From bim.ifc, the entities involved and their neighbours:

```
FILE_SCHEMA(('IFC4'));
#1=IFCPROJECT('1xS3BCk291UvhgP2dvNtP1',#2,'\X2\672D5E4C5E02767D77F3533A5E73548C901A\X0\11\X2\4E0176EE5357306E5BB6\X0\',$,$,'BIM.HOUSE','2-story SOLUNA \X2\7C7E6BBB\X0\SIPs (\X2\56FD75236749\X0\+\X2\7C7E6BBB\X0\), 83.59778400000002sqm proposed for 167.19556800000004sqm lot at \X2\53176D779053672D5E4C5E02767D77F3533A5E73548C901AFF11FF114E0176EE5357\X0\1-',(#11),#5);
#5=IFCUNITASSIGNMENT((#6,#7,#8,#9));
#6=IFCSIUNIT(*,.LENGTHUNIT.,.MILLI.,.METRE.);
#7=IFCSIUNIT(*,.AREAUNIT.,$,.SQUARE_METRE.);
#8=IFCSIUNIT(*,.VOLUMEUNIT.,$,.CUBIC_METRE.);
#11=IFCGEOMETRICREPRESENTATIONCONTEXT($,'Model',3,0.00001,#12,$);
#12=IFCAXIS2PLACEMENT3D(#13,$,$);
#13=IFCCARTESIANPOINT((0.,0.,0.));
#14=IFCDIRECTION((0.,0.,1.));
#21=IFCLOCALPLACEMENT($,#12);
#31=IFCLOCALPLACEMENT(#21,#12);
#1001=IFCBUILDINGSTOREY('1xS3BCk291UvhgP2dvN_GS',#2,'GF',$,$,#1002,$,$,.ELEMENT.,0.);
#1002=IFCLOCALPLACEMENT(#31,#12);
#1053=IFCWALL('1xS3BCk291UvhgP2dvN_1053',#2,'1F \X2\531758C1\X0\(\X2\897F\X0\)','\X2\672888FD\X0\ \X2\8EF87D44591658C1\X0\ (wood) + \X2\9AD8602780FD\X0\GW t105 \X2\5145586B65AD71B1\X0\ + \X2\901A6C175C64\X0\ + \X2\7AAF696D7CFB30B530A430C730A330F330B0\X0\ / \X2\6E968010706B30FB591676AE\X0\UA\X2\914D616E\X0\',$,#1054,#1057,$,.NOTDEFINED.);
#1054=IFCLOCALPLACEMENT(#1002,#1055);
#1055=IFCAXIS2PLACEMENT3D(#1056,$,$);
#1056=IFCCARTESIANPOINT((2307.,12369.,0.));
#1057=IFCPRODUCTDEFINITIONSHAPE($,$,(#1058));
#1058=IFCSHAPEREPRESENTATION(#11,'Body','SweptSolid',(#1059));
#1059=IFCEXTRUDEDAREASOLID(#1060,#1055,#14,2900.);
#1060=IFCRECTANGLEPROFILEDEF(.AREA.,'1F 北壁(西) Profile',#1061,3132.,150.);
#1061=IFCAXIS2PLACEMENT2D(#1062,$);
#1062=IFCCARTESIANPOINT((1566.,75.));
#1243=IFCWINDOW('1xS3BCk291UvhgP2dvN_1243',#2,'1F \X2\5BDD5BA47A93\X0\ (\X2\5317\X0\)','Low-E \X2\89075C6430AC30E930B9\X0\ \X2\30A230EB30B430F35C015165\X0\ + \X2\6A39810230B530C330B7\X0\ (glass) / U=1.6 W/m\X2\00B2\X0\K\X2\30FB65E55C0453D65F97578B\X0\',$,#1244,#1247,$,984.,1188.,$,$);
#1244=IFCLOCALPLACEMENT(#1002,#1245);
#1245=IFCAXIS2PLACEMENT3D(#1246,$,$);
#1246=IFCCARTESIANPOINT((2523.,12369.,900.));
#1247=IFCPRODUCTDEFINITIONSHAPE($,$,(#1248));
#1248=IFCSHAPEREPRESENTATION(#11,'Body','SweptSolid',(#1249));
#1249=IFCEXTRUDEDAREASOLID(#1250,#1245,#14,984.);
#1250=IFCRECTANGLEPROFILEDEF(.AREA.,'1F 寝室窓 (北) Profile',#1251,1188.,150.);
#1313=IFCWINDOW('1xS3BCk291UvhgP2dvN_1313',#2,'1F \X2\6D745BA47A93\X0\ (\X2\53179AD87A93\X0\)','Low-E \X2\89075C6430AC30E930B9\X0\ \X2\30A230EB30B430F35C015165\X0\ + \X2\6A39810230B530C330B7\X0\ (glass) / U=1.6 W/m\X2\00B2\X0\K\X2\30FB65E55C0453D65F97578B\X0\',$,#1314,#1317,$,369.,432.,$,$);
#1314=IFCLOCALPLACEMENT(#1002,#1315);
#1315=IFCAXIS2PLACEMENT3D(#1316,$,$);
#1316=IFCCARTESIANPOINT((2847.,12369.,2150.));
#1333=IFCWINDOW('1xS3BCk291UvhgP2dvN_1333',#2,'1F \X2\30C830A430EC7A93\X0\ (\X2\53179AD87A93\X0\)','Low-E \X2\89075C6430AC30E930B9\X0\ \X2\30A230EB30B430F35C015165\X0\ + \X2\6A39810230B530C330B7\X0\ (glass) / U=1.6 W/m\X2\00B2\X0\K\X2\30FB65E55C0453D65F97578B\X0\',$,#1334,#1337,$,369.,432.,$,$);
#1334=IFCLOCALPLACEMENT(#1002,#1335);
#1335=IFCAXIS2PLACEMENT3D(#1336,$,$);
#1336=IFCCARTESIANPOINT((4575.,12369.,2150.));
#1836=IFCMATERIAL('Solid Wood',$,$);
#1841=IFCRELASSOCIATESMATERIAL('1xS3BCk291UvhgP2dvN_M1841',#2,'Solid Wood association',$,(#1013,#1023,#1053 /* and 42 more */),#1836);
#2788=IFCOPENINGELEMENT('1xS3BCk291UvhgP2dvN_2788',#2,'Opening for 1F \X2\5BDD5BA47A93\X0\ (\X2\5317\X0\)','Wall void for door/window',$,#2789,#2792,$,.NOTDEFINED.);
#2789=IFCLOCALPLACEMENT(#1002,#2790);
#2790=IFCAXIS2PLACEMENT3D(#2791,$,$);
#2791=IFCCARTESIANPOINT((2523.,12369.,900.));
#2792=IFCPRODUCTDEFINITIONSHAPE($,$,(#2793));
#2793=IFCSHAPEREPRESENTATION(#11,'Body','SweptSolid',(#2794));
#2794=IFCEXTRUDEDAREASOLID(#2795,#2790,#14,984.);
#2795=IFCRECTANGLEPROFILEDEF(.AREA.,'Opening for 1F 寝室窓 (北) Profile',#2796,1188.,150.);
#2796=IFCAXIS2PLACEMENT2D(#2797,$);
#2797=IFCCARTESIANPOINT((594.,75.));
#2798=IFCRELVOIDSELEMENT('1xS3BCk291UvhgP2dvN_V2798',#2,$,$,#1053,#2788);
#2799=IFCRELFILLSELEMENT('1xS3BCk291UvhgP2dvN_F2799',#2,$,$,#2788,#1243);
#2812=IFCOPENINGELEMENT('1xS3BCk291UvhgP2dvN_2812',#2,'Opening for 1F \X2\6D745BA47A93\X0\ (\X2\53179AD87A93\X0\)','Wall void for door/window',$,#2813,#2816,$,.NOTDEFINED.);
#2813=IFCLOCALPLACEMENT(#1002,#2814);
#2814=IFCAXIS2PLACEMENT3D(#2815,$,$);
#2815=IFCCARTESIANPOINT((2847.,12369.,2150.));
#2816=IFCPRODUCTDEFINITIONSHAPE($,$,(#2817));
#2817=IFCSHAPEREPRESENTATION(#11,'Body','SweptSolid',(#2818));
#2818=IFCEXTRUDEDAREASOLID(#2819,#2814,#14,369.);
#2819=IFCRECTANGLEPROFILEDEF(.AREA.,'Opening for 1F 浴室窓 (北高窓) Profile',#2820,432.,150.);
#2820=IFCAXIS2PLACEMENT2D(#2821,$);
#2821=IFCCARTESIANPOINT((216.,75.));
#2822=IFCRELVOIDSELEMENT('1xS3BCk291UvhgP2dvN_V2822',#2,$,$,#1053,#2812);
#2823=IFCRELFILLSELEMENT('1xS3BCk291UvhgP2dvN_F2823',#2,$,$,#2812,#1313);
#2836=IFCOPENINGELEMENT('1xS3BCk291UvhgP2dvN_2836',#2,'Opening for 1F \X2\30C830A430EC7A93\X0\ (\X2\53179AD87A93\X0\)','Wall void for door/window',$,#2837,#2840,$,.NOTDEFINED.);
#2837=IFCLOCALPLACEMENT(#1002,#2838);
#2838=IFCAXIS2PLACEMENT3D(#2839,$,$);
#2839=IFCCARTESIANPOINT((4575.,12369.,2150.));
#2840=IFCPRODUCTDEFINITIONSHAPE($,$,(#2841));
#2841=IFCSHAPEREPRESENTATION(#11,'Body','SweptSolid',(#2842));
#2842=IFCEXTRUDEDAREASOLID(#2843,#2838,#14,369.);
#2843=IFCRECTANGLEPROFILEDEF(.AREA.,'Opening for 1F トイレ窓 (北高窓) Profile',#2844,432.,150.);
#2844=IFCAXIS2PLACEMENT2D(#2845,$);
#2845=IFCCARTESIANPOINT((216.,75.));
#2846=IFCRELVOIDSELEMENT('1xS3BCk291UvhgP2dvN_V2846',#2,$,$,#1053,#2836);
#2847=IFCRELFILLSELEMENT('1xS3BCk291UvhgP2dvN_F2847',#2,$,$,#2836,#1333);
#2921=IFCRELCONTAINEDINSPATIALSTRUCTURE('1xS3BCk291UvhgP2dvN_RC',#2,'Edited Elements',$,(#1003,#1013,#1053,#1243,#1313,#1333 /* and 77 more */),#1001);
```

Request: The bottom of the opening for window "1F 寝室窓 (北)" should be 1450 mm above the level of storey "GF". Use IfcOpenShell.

```python
import numpy as np
import ifcopenshell
import ifcopenshell.api.geometry
import ifcopenshell.geom
import ifcopenshell.util.element
import ifcopenshell.util.placement
import ifcopenshell.util.shape
import ifcopenshell.util.unit

model = ifcopenshell.open("bim.ifc")
unit_scale = ifcopenshell.util.unit.calculate_unit_scale(model)

window = model.by_id(1243)
opening = window.FillsVoids[0].RelatingOpeningElement
storey = ifcopenshell.util.element.get_container(window, ifc_class="IfcBuildingStorey")
level = ifcopenshell.util.placement.get_local_placement(storey.ObjectPlacement)[2, 3]

# The opening's origin need not be at the sill, so measure its lowest point.
shape = ifcopenshell.geom.create_shape(ifcopenshell.geom.settings(), opening)
bottom = ifcopenshell.util.shape.get_shape_bottom_elevation(shape, shape.geometry) / unit_scale
dz = level + 1450.0 - bottom

shift = np.array([0.0, 0.0, dz])
# The window is not placed relative to its opening, so move both.
for product in (opening, window):
    matrix = ifcopenshell.util.placement.get_local_placement(product.ObjectPlacement)
    matrix[:3, 3] += shift
    ifcopenshell.api.geometry.edit_object_placement(model, product=product, matrix=matrix, is_si=False)

print(f"moved by {dz * unit_scale:+.3f} m")

model.write("bim_v2.ifc")
```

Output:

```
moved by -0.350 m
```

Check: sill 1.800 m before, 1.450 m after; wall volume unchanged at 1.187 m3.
